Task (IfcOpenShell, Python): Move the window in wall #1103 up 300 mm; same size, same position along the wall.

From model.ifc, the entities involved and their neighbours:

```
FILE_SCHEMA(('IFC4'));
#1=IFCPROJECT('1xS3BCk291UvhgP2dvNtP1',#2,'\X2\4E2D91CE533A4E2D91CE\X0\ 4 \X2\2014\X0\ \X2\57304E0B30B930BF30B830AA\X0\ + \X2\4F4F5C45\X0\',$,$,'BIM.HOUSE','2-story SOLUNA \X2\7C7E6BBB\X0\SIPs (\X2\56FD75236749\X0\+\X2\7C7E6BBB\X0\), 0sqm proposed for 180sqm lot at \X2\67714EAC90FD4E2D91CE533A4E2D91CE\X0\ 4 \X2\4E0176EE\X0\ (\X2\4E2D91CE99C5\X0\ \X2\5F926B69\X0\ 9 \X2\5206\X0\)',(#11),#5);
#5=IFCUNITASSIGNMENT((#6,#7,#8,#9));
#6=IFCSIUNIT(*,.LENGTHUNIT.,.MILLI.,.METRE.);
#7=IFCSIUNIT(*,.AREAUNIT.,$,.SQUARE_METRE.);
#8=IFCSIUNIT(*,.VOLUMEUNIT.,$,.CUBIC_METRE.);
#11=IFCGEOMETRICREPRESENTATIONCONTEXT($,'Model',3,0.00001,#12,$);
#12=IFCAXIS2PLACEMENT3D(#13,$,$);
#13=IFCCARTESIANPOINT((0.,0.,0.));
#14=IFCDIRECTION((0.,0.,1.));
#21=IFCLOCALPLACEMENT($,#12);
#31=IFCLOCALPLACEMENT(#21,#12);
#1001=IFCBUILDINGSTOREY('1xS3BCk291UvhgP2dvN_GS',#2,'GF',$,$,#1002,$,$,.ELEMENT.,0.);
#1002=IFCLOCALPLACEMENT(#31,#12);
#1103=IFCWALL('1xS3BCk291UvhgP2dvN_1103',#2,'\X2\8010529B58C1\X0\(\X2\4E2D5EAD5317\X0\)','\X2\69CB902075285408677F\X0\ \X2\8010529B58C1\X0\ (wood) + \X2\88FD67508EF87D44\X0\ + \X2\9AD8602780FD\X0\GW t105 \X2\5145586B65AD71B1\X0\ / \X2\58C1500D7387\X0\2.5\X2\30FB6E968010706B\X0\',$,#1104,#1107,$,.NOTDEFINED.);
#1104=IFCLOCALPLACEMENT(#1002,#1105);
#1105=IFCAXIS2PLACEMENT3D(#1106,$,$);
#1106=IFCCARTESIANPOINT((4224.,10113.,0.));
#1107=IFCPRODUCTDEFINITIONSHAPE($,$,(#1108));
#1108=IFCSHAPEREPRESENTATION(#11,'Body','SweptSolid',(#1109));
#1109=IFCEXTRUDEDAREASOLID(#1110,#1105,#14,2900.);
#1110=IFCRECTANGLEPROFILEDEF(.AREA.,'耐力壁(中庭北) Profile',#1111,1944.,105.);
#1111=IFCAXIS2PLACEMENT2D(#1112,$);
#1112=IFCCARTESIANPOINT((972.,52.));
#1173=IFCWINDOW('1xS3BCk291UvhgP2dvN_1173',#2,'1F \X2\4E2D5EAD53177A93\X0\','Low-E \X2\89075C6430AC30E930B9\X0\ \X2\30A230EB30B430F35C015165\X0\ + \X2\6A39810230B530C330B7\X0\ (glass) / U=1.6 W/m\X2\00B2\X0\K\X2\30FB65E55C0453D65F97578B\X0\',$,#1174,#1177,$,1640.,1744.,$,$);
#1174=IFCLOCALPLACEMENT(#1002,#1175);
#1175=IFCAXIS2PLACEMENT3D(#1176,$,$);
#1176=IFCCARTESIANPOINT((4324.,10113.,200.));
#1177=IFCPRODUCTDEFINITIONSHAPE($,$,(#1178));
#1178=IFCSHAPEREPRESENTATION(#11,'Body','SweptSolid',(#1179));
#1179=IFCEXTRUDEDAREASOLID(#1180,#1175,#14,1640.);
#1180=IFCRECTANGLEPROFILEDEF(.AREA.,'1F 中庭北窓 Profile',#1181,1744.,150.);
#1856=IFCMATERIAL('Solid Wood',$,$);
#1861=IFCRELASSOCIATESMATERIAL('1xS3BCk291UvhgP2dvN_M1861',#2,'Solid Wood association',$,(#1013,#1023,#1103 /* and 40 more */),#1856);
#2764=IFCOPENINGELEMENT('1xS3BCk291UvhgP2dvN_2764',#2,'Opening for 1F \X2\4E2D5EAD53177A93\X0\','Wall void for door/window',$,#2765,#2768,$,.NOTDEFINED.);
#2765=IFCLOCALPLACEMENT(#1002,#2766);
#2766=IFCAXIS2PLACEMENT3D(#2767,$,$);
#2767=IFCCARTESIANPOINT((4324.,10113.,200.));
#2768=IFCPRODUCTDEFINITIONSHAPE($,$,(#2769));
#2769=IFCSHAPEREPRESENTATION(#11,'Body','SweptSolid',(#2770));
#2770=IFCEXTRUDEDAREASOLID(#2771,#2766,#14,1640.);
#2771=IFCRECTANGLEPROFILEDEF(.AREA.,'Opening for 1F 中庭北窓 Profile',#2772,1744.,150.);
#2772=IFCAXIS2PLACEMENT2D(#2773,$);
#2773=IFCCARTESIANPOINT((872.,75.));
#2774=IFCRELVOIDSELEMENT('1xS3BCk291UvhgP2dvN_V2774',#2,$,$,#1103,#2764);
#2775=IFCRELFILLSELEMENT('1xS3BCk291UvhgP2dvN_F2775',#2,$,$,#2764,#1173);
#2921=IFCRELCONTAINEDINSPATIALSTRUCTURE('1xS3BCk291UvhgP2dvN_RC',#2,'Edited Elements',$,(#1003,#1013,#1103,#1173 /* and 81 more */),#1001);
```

```python
import numpy as np
import ifcopenshell
import ifcopenshell.api.geometry
import ifcopenshell.util.placement
import ifcopenshell.util.unit

model = ifcopenshell.open("model.ifc")
unit_scale = ifcopenshell.util.unit.calculate_unit_scale(model)

window = model.by_guid("1xS3BCk291UvhgP2dvN_1173")
opening = window.FillsVoids[0].RelatingOpeningElement
dz = 300.0

shift = np.array([0.0, 0.0, dz])
# The window is not placed relative to its opening, so move both.
for product in (opening, window):
    matrix = ifcopenshell.util.placement.get_local_placement(product.ObjectPlacement)
    matrix[:3, 3] += shift
    ifcopenshell.api.geometry.edit_object_placement(model, product=product, matrix=matrix, is_si=False)

print(f"moved by {dz * unit_scale:+.3f} m")

model.write("model_updated.ifc")
```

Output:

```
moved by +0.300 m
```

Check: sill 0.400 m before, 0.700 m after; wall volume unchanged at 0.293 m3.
